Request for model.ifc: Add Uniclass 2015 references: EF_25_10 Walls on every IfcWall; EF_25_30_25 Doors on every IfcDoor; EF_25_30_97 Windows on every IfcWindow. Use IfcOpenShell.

First a look at what the model holds.

```python
import ifcopenshell

model = ifcopenshell.open("model.ifc")
print(model.schema)
print("classifications:", [c.Name for c in model.by_type("IfcClassification")])
for ifc_class in ("IfcDoor", "IfcRoof", "IfcStair", "IfcWall", "IfcWindow"):
    print(ifc_class, len(model.by_type(ifc_class)))
```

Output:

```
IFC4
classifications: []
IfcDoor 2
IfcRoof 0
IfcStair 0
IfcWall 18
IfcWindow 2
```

```python
import ifcopenshell
import ifcopenshell.api.classification

model = ifcopenshell.open("model.ifc")

system = ifcopenshell.api.classification.add_classification(model, classification="Uniclass 2015")

codes = {
    "IfcWall": ("EF_25_10", "Walls"),
    "IfcDoor": ("EF_25_30_25", "Doors"),
    "IfcWindow": ("EF_25_30_97", "Windows"),
}
for ifc_class, (code, name) in codes.items():
    products = model.by_type(ifc_class)
    ifcopenshell.api.classification.add_reference(
        model, products=products, classification=system, identification=code, name=name
    )
    print(code, len(products))

model.write("model-out.ifc")
```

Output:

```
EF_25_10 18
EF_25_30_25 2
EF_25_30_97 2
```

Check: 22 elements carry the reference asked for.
